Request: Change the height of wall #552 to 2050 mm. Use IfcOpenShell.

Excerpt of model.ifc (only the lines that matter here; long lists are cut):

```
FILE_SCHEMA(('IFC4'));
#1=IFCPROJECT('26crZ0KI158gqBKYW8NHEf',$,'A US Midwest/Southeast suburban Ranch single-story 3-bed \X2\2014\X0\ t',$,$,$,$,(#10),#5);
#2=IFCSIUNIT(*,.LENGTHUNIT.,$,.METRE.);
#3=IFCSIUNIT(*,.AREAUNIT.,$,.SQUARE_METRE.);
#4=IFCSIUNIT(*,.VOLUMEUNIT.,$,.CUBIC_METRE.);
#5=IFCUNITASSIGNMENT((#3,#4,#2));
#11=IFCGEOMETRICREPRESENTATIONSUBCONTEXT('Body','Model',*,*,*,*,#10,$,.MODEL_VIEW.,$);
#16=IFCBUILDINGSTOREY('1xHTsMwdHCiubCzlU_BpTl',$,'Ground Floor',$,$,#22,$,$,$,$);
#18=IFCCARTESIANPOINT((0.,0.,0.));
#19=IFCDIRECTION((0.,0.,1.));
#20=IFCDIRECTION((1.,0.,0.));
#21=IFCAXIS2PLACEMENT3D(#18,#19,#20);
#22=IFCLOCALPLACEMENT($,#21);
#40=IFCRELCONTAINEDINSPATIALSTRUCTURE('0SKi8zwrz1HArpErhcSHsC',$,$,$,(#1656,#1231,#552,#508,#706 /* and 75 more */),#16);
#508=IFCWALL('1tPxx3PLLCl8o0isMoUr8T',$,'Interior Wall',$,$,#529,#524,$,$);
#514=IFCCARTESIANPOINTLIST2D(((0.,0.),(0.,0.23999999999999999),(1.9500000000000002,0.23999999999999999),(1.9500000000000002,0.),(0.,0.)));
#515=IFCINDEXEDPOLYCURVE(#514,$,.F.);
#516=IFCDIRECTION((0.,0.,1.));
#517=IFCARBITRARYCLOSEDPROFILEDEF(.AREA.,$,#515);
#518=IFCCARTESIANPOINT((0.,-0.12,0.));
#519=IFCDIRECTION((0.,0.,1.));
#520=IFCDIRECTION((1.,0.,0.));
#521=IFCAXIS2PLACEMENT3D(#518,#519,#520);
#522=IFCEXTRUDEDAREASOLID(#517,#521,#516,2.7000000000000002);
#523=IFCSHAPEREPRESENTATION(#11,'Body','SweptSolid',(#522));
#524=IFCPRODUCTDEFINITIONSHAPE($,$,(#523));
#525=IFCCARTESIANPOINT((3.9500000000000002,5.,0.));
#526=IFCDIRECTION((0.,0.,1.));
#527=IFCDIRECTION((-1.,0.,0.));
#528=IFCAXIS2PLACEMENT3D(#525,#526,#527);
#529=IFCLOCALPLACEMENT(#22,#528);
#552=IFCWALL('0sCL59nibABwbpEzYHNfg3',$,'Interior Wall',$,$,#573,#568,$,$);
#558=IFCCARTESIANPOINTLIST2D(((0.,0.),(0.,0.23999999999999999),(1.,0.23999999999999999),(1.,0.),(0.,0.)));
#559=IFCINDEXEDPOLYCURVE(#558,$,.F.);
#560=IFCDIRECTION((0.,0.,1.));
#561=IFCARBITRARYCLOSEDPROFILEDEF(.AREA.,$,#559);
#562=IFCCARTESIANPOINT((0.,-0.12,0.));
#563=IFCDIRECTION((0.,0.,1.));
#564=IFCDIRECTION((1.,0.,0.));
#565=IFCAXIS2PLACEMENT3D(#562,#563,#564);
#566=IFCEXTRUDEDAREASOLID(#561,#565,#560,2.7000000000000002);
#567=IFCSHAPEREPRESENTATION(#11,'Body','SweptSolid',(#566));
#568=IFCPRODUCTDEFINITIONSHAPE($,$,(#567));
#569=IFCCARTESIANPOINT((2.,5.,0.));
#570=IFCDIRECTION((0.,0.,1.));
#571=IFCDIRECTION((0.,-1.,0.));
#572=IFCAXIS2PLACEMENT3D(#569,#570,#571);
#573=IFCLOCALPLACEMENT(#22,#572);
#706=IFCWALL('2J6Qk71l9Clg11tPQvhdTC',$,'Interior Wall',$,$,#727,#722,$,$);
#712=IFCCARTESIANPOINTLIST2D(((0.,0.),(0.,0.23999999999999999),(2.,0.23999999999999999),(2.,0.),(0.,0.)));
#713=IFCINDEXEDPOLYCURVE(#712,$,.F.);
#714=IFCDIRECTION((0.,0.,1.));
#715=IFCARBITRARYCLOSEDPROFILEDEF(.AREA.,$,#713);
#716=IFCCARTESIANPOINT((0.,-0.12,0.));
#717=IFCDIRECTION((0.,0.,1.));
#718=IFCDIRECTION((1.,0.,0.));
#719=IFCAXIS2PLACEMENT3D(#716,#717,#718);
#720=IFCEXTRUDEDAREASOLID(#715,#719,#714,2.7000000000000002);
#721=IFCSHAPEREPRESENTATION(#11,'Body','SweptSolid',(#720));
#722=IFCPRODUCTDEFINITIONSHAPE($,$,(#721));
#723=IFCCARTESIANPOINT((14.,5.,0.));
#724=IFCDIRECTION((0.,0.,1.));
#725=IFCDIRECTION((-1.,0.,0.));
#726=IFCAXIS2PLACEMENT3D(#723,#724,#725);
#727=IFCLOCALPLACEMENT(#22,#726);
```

```python
import ifcopenshell
import ifcopenshell.geom
import ifcopenshell.util.representation
import ifcopenshell.util.shape
import ifcopenshell.util.unit

model = ifcopenshell.open("model.ifc")
unit_scale = ifcopenshell.util.unit.calculate_unit_scale(model)
settings = ifcopenshell.geom.settings()


def volume(element):
    """Net volume in cubic metres, openings subtracted."""
    shape = ifcopenshell.geom.create_shape(settings, element)
    return ifcopenshell.util.shape.get_volume(shape.geometry)


wall = model.by_id(552)
before = volume(wall)

body = ifcopenshell.util.representation.get_representation(wall, "Model", "Body")
solid = body.Items[0]
old_height = solid.Depth
solid.Depth = 2.05 / unit_scale
after = volume(wall)

print(f"height {old_height:g} -> {solid.Depth:g}, volume {before:.3f} -> {after:.3f} m3")

model.write("model-out.ifc")
```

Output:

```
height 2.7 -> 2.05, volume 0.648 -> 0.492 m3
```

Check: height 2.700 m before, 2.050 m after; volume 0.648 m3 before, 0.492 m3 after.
